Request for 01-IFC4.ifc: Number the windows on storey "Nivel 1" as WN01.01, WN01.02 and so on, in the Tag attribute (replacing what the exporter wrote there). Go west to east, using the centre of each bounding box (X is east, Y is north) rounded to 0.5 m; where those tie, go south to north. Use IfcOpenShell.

First a look at what the model holds.

```python
import ifcopenshell
import ifcopenshell.util.element
import ifcopenshell.util.placement

model = ifcopenshell.open("01-IFC4.ifc")
print(model.schema)
storey = next(s for s in model.by_type("IfcBuildingStorey") if s.Name == "Nivel 1")
windows = [e for e in ifcopenshell.util.element.get_decomposition(storey) if e.is_a("IfcWindow")]
for e in sorted(windows, key=lambda e: e.id()):
    origin = ifcopenshell.util.placement.get_local_placement(e.ObjectPlacement)[:3, 3]
    print(e.id(), e.Tag, e.Name, origin.round(2) + 0.0, sep=" | ")
```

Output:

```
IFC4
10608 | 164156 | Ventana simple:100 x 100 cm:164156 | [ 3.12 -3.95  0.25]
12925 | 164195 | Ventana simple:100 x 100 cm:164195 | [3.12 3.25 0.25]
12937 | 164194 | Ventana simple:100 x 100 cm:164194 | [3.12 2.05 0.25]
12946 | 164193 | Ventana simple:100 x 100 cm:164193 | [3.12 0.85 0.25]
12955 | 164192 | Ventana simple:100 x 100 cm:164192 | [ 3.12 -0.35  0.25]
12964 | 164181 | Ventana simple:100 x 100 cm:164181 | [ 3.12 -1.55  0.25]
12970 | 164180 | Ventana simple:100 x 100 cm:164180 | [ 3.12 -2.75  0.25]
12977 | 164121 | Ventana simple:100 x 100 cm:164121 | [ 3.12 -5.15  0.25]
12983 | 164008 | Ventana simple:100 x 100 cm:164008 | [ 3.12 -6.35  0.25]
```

```python
import ifcopenshell
import ifcopenshell.geom
import ifcopenshell.util.element
import ifcopenshell.util.shape

model = ifcopenshell.open("01-IFC4.ifc")
settings = ifcopenshell.geom.settings()
settings.set("use-world-coords", True)


def centre(element):
    shape = ifcopenshell.geom.create_shape(settings, element)
    return ifcopenshell.util.shape.get_bbox_centroid(shape.geometry)


storey = next(s for s in model.by_type("IfcBuildingStorey") if s.Name == "Nivel 1")
windows = [e for e in ifcopenshell.util.element.get_decomposition(storey) if e.is_a("IfcWindow")]

# Insertion points can sit at a corner or the storey origin, so sort by the geometry (in metres).
centres = {e: centre(e) for e in windows}
windows.sort(key=lambda e: (round(centres[e][0] / 0.5), centres[e][1]))

for i, e in enumerate(windows, start=1):
    number = f"WN01.{i:02d}"
    e.Tag = number
    print(e.id(), number)

model.write("01-IFC4_edited.ifc")
```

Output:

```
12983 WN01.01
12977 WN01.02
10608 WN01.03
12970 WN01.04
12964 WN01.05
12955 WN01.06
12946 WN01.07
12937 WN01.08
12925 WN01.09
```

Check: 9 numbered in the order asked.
